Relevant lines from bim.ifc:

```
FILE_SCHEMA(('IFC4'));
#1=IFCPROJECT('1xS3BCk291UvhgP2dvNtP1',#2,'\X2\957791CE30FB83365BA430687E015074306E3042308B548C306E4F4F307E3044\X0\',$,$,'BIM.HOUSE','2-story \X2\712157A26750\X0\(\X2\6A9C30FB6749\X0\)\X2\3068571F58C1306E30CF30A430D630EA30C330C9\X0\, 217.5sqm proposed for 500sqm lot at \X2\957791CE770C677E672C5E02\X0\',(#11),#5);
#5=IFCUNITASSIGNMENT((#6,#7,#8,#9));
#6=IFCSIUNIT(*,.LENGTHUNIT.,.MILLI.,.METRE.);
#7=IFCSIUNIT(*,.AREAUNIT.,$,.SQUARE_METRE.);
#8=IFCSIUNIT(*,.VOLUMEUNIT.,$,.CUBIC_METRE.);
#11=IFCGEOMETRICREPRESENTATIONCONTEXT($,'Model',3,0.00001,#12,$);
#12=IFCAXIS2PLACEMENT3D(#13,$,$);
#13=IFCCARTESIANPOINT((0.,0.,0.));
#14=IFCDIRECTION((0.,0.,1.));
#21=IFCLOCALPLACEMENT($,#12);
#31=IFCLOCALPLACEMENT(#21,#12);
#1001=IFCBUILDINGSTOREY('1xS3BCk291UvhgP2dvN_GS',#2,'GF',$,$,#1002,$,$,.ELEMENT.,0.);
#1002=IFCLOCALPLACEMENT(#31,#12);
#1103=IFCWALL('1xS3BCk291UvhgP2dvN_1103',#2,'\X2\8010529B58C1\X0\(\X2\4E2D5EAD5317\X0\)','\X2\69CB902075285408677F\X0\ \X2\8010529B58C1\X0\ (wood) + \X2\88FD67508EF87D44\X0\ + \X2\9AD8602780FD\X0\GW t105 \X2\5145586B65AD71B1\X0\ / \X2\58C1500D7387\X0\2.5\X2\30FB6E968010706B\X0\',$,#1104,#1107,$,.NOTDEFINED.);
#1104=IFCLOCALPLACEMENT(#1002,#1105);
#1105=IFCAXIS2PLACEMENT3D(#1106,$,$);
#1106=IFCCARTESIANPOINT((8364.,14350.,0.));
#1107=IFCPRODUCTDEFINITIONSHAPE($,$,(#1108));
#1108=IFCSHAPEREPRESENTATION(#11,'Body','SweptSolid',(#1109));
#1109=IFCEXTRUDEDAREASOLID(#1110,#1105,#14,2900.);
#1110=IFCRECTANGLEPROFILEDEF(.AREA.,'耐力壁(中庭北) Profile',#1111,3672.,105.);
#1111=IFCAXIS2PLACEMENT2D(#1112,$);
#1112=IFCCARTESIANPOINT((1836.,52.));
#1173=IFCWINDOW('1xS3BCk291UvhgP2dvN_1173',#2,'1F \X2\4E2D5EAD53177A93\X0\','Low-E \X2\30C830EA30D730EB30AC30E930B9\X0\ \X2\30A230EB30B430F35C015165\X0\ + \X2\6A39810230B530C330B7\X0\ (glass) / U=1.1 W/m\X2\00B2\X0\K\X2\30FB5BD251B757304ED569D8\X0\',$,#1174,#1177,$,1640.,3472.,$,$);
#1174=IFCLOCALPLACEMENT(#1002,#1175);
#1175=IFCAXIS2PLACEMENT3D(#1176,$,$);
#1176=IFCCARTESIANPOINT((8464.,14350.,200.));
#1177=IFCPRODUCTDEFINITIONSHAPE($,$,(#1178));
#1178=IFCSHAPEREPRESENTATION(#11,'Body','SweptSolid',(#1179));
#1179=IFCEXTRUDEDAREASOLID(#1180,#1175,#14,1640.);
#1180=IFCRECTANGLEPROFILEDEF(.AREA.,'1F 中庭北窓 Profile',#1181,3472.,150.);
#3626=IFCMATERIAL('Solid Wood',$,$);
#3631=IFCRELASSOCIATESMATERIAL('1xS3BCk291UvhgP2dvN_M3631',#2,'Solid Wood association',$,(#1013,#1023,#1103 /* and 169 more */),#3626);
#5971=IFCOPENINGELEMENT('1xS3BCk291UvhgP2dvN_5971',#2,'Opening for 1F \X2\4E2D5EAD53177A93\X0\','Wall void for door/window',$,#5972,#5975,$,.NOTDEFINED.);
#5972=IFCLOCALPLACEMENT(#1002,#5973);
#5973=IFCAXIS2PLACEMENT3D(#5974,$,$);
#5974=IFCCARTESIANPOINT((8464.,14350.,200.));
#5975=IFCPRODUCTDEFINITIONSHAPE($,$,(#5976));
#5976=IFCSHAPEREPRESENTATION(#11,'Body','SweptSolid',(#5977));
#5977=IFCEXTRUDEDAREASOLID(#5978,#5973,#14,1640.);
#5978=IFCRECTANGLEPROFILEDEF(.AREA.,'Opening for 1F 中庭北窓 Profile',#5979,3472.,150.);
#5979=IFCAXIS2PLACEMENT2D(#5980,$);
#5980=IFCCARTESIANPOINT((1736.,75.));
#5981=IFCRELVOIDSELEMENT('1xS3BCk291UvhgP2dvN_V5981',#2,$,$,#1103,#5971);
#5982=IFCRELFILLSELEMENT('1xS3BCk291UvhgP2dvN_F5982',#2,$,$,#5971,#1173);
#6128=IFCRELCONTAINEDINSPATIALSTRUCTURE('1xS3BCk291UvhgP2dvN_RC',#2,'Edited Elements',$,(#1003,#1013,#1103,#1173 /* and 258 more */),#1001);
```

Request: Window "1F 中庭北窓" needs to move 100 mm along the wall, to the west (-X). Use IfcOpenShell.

```python
import ifcopenshell
import ifcopenshell.api.geometry
import ifcopenshell.util.placement

model = ifcopenshell.open("bim.ifc")

window = model.by_guid("1xS3BCk291UvhgP2dvN_1173")
opening = window.FillsVoids[0].RelatingOpeningElement
wall = opening.VoidsElements[0].RelatingBuildingElement

wall_matrix = ifcopenshell.util.placement.get_local_placement(wall.ObjectPlacement)
shift = wall_matrix[:3, 0] * -100.0
before = ifcopenshell.util.placement.get_local_placement(window.ObjectPlacement)[:3, 3].copy()

# The window is not placed relative to its opening, so move both.
for product in (opening, window):
    matrix = ifcopenshell.util.placement.get_local_placement(product.ObjectPlacement)
    matrix[:3, 3] += shift
    ifcopenshell.api.geometry.edit_object_placement(model, product=product, matrix=matrix, is_si=False)

after = ifcopenshell.util.placement.get_local_placement(window.ObjectPlacement)[:3, 3]
print("window moved by", (after - before).round(3) + 0.0)

model.write("bim_updated.ifc")
```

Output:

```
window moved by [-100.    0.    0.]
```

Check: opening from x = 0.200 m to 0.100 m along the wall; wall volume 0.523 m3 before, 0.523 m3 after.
